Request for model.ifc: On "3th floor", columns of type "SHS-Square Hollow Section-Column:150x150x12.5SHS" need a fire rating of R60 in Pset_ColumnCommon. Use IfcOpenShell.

First a look at what the model holds.

```python
import ifcopenshell
import ifcopenshell.util.element

model = ifcopenshell.open("model.ifc")
print(model.schema)
storey = next(s for s in model.by_type("IfcBuildingStorey") if s.Name == "3th floor")
columns = [e for e in ifcopenshell.util.element.get_decomposition(storey) if e.is_a("IfcColumn")]
seen = {}
for e in columns:
    element_type = ifcopenshell.util.element.get_type(e)
    key = (element_type.Name if element_type != e and element_type else None, ifcopenshell.util.element.get_pset(e, "Pset_ColumnCommon", "FireRating"))
    seen[key] = seen.get(key, 0) + 1
for (name, value), count in sorted(seen.items(), key=str):
    print(count, "x", name, "|", value)
```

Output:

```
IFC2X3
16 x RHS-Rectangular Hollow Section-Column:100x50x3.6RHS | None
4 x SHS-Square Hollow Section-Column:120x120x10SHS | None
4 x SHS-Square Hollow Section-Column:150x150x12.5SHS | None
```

```python
import ifcopenshell
import ifcopenshell.api.pset
import ifcopenshell.util.element

model = ifcopenshell.open("model.ifc")

storey = next(s for s in model.by_type("IfcBuildingStorey") if s.Name == "3th floor")
columns = [e for e in ifcopenshell.util.element.get_decomposition(storey) if e.is_a("IfcColumn")]

count = 0
for e in columns:
    element_type = ifcopenshell.util.element.get_type(e)
    if element_type in (None, e) or element_type.Name != "SHS-Square Hollow Section-Column:150x150x12.5SHS":
        continue
    # add_pset returns the element's existing set when there is one.
    pset = ifcopenshell.api.pset.add_pset(model, product=e, name="Pset_ColumnCommon")
    ifcopenshell.api.pset.edit_pset(model, pset=pset, properties={"FireRating": "R60"})
    count += 1

print(count, "columns updated")

model.write("model_edited.ifc")
```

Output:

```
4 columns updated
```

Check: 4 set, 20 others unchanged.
